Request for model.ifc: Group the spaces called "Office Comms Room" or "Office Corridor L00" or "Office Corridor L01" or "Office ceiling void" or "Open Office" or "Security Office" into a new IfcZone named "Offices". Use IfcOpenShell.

First a look at what the model holds.

```python
import ifcopenshell

model = ifcopenshell.open("model.ifc")
print(model.schema)
seen = {}
for space in model.by_type("IfcSpace"):
    seen[space.LongName] = seen.get(space.LongName, 0) + 1
for name, count in sorted(seen.items(), key=str):
    print(count, "x", name)
print("zones:", [z.Name for z in model.by_type("IfcZone")][:20])
```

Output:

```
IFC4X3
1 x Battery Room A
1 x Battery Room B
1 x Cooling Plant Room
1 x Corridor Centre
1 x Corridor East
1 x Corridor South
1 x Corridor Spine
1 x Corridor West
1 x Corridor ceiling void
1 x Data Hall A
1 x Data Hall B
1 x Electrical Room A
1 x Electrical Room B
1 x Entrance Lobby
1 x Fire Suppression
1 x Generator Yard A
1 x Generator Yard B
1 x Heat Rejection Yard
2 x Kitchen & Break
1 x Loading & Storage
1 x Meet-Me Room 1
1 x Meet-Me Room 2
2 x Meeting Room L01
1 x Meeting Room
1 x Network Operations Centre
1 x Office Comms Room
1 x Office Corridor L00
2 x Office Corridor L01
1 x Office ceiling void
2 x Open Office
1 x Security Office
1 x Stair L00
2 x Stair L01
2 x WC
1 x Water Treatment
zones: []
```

```python
import ifcopenshell
import ifcopenshell.api.group
import ifcopenshell.api.root

model = ifcopenshell.open("model.ifc")

names = {"Office Comms Room", "Office Corridor L00", "Office Corridor L01", "Office ceiling void", "Open Office", "Security Office"}
spaces = [s for s in model.by_type("IfcSpace") if s.LongName in names]

zone = ifcopenshell.api.root.create_entity(model, ifc_class="IfcZone", name="Offices")
ifcopenshell.api.group.assign_group(model, products=spaces, group=zone)
print(len(spaces), "spaces in", zone.Name)

model.write("model_updated.ifc")
```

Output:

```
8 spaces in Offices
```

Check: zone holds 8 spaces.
